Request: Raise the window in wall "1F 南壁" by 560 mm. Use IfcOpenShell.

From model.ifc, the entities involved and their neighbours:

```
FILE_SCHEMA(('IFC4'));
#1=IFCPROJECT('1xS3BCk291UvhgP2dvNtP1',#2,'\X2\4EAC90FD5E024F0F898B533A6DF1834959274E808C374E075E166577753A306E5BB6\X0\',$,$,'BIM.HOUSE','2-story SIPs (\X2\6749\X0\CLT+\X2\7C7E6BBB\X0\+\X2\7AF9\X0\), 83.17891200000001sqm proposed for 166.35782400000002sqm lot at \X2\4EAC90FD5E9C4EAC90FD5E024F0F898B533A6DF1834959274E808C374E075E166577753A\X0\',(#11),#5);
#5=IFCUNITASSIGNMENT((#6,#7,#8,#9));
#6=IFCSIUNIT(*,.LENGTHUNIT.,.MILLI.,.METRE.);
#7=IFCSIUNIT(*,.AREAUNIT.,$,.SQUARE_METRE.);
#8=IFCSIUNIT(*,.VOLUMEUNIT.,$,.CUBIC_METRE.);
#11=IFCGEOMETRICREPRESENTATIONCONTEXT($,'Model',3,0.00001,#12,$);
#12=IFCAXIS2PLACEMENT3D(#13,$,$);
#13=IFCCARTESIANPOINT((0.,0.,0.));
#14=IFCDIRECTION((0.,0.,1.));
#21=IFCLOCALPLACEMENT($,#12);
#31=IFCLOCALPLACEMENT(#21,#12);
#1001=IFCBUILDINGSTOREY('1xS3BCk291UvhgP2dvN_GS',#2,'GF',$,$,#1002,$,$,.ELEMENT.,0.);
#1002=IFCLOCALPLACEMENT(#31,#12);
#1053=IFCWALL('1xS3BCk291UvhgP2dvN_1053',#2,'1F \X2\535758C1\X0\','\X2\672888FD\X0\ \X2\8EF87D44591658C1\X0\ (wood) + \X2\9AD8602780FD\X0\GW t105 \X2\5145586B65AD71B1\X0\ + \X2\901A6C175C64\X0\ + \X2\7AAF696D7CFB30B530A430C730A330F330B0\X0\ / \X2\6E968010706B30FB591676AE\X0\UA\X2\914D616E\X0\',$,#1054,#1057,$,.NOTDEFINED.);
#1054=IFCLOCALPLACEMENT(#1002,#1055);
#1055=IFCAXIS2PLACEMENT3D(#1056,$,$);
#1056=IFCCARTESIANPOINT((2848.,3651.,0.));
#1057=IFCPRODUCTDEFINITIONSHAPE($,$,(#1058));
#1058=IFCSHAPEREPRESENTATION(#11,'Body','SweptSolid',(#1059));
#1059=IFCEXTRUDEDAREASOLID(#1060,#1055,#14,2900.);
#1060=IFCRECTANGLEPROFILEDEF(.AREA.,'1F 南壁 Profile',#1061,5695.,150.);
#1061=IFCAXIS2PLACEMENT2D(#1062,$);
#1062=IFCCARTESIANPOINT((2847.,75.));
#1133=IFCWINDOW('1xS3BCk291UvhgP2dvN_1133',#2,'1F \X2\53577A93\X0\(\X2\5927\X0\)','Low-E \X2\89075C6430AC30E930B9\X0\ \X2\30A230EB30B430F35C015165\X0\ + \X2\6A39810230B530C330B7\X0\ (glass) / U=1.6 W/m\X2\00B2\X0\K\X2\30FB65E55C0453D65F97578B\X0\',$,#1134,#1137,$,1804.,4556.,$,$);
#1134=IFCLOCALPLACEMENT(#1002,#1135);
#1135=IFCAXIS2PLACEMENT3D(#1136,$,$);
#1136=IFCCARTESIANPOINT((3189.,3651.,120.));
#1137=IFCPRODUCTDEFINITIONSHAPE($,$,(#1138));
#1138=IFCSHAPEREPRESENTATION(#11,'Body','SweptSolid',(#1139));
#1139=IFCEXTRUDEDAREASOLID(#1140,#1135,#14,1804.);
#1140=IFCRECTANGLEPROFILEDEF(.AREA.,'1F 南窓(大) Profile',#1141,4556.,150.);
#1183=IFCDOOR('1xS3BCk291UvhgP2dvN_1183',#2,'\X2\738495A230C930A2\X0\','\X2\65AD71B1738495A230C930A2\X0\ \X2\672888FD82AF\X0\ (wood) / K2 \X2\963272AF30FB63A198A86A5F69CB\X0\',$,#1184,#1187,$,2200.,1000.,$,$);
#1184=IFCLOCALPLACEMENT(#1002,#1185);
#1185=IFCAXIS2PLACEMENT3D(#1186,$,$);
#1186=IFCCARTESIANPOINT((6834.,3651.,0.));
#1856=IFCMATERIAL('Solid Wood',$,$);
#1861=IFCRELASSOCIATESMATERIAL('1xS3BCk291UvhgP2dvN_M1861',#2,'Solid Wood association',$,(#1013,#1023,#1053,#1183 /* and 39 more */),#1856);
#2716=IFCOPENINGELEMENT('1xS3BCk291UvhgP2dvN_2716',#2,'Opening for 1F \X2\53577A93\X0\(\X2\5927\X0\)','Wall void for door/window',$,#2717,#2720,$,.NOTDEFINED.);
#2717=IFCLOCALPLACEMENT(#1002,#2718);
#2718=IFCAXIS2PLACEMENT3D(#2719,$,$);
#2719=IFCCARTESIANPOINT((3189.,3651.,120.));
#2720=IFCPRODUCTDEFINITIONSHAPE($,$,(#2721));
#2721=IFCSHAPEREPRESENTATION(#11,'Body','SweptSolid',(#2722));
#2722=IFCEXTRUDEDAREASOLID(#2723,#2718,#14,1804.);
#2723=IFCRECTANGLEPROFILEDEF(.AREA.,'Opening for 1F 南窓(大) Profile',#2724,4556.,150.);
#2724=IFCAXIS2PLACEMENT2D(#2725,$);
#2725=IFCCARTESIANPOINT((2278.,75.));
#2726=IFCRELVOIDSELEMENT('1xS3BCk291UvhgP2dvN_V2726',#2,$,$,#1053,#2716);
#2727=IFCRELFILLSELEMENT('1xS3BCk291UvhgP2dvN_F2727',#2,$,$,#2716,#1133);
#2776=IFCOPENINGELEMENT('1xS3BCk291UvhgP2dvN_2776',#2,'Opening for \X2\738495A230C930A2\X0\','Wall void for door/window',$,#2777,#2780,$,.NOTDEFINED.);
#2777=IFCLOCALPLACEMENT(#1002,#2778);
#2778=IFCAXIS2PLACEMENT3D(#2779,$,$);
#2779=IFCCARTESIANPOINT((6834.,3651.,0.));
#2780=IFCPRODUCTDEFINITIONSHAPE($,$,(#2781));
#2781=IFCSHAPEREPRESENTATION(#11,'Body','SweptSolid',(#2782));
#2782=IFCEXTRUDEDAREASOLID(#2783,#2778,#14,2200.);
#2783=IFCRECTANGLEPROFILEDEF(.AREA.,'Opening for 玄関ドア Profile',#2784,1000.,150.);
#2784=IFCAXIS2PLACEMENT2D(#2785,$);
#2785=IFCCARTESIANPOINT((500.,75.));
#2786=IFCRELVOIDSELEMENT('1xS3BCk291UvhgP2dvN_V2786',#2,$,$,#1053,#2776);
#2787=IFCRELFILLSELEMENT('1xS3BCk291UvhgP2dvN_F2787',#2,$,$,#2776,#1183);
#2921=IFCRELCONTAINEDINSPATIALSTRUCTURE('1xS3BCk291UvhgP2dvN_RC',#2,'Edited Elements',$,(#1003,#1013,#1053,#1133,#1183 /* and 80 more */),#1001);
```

```python
import numpy as np
import ifcopenshell
import ifcopenshell.api.geometry
import ifcopenshell.util.placement
import ifcopenshell.util.unit

model = ifcopenshell.open("model.ifc")
unit_scale = ifcopenshell.util.unit.calculate_unit_scale(model)

window = model.by_id(1133)
opening = window.FillsVoids[0].RelatingOpeningElement
dz = 560.0

shift = np.array([0.0, 0.0, dz])
# The window is not placed relative to its opening, so move both.
for product in (opening, window):
    matrix = ifcopenshell.util.placement.get_local_placement(product.ObjectPlacement)
    matrix[:3, 3] += shift
    ifcopenshell.api.geometry.edit_object_placement(model, product=product, matrix=matrix, is_si=False)

print(f"moved by {dz * unit_scale:+.3f} m")

model.write("model_rev.ifc")
```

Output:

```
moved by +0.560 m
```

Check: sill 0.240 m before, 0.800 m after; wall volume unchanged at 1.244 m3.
